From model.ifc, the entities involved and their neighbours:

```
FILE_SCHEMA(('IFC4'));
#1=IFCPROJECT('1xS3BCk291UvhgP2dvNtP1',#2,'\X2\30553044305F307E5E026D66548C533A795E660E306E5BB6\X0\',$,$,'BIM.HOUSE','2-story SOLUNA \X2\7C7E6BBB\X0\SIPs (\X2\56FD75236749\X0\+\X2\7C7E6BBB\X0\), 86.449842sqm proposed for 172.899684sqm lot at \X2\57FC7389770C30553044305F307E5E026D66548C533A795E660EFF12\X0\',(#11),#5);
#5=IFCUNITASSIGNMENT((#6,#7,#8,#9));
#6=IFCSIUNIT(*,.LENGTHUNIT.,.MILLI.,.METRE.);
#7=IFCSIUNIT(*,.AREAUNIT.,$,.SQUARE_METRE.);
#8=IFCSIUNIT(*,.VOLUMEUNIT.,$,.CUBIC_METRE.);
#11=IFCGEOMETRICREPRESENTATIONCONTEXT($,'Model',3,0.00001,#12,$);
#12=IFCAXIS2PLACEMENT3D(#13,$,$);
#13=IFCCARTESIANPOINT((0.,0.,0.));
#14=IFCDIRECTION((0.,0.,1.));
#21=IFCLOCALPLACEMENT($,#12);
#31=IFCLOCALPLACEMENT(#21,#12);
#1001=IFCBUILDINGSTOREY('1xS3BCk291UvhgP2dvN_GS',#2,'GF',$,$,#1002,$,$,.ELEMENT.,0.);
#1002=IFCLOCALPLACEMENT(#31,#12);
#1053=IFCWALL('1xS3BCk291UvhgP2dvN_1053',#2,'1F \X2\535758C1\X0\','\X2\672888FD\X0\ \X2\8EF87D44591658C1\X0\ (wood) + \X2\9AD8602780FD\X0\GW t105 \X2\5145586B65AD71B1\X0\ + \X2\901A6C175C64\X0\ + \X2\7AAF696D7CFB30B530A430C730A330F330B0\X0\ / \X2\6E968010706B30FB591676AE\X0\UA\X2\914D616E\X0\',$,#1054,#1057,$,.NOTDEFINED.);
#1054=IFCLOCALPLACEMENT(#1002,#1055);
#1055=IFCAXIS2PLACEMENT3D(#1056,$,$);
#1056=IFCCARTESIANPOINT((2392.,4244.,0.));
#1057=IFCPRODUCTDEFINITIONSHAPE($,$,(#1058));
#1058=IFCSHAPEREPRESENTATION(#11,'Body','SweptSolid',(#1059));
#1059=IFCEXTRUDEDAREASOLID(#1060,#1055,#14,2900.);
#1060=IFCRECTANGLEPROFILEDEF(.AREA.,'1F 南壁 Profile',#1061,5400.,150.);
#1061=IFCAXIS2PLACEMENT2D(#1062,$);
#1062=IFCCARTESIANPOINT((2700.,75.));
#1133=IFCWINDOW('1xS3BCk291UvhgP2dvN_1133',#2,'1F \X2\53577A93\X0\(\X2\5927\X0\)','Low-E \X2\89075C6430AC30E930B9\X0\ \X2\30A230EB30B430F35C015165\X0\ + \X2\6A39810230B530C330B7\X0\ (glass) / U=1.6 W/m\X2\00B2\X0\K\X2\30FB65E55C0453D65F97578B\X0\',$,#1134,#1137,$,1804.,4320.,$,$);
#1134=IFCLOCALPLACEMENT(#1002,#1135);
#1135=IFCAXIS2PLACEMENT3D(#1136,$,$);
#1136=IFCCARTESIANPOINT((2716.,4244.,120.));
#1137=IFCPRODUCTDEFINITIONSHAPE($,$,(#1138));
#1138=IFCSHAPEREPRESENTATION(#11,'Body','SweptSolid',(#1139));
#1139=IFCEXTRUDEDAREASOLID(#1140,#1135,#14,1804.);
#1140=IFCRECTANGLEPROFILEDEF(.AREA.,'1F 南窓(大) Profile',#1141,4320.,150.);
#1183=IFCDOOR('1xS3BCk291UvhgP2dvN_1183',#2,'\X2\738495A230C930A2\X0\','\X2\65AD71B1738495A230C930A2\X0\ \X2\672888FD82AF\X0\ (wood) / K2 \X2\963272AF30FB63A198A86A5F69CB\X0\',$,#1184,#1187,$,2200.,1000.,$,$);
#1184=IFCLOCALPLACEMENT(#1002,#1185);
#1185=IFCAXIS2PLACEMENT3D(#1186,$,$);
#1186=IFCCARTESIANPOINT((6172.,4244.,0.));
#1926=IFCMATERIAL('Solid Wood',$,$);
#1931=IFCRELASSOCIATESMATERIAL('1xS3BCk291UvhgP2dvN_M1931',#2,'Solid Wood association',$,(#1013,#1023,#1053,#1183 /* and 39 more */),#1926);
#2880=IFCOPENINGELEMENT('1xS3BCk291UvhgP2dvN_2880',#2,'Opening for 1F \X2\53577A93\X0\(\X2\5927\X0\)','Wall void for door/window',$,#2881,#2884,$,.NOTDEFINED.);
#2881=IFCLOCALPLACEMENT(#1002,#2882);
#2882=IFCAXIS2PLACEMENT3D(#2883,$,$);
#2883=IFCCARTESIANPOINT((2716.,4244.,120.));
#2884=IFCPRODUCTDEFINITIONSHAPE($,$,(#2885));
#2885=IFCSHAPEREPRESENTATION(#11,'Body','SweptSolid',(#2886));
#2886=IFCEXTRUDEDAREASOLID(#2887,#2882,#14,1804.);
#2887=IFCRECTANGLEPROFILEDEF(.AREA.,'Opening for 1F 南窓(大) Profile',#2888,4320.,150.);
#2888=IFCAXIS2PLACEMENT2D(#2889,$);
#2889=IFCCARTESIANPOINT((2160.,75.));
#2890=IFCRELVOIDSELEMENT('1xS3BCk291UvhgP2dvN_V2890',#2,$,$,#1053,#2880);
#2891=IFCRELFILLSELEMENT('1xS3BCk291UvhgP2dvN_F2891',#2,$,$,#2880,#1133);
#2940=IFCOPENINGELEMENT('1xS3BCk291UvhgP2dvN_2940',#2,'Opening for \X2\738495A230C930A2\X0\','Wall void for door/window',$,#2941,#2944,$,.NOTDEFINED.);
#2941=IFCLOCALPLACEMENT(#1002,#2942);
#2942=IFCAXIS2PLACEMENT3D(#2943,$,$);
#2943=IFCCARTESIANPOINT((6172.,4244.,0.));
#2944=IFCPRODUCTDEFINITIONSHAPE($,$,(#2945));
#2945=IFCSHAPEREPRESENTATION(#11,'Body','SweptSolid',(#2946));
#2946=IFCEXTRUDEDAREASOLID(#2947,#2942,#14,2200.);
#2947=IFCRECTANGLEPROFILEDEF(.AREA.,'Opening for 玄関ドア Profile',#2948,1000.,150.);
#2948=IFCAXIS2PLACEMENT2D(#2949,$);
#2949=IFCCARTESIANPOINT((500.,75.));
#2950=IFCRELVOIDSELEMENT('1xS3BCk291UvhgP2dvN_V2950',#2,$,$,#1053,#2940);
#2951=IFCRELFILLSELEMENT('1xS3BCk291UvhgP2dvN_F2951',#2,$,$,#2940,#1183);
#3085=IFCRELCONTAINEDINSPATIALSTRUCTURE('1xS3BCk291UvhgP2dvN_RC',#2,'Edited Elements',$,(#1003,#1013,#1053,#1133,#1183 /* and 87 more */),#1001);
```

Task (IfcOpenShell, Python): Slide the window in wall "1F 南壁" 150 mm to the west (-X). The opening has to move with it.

```python
import ifcopenshell
import ifcopenshell.api.geometry
import ifcopenshell.util.placement

model = ifcopenshell.open("model.ifc")

window = model.by_guid("1xS3BCk291UvhgP2dvN_1133")
opening = window.FillsVoids[0].RelatingOpeningElement
wall = opening.VoidsElements[0].RelatingBuildingElement

wall_matrix = ifcopenshell.util.placement.get_local_placement(wall.ObjectPlacement)
shift = wall_matrix[:3, 0] * -150.0
before = ifcopenshell.util.placement.get_local_placement(window.ObjectPlacement)[:3, 3].copy()

# The window is not placed relative to its opening, so move both.
for product in (opening, window):
    matrix = ifcopenshell.util.placement.get_local_placement(product.ObjectPlacement)
    matrix[:3, 3] += shift
    ifcopenshell.api.geometry.edit_object_placement(model, product=product, matrix=matrix, is_si=False)

after = ifcopenshell.util.placement.get_local_placement(window.ObjectPlacement)[:3, 3]
print("window moved by", (after - before).round(3) + 0.0)

model.write("model_rev.ifc")
```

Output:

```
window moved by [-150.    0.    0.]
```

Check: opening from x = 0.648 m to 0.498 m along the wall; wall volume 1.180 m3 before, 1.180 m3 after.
